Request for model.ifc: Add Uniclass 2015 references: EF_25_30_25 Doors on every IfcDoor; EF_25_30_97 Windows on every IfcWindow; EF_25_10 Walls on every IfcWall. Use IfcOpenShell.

First a look at what the model holds.

```python
import ifcopenshell

model = ifcopenshell.open("model.ifc")
print(model.schema)
print("classifications:", [c.Name for c in model.by_type("IfcClassification")])
for ifc_class in ("IfcDoor", "IfcRoof", "IfcStair", "IfcWall", "IfcWindow"):
    print(ifc_class, len(model.by_type(ifc_class)))
```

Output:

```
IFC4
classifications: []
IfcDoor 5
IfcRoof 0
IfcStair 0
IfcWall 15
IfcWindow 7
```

```python
import ifcopenshell
import ifcopenshell.api.classification

model = ifcopenshell.open("model.ifc")

system = ifcopenshell.api.classification.add_classification(model, classification="Uniclass 2015")

codes = {
    "IfcDoor": ("EF_25_30_25", "Doors"),
    "IfcWindow": ("EF_25_30_97", "Windows"),
    "IfcWall": ("EF_25_10", "Walls"),
}
for ifc_class, (code, name) in codes.items():
    products = model.by_type(ifc_class)
    ifcopenshell.api.classification.add_reference(
        model, products=products, classification=system, identification=code, name=name
    )
    print(code, len(products))

model.write("model_updated.ifc")
```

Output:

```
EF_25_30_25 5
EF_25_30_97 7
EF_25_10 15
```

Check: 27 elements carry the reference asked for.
